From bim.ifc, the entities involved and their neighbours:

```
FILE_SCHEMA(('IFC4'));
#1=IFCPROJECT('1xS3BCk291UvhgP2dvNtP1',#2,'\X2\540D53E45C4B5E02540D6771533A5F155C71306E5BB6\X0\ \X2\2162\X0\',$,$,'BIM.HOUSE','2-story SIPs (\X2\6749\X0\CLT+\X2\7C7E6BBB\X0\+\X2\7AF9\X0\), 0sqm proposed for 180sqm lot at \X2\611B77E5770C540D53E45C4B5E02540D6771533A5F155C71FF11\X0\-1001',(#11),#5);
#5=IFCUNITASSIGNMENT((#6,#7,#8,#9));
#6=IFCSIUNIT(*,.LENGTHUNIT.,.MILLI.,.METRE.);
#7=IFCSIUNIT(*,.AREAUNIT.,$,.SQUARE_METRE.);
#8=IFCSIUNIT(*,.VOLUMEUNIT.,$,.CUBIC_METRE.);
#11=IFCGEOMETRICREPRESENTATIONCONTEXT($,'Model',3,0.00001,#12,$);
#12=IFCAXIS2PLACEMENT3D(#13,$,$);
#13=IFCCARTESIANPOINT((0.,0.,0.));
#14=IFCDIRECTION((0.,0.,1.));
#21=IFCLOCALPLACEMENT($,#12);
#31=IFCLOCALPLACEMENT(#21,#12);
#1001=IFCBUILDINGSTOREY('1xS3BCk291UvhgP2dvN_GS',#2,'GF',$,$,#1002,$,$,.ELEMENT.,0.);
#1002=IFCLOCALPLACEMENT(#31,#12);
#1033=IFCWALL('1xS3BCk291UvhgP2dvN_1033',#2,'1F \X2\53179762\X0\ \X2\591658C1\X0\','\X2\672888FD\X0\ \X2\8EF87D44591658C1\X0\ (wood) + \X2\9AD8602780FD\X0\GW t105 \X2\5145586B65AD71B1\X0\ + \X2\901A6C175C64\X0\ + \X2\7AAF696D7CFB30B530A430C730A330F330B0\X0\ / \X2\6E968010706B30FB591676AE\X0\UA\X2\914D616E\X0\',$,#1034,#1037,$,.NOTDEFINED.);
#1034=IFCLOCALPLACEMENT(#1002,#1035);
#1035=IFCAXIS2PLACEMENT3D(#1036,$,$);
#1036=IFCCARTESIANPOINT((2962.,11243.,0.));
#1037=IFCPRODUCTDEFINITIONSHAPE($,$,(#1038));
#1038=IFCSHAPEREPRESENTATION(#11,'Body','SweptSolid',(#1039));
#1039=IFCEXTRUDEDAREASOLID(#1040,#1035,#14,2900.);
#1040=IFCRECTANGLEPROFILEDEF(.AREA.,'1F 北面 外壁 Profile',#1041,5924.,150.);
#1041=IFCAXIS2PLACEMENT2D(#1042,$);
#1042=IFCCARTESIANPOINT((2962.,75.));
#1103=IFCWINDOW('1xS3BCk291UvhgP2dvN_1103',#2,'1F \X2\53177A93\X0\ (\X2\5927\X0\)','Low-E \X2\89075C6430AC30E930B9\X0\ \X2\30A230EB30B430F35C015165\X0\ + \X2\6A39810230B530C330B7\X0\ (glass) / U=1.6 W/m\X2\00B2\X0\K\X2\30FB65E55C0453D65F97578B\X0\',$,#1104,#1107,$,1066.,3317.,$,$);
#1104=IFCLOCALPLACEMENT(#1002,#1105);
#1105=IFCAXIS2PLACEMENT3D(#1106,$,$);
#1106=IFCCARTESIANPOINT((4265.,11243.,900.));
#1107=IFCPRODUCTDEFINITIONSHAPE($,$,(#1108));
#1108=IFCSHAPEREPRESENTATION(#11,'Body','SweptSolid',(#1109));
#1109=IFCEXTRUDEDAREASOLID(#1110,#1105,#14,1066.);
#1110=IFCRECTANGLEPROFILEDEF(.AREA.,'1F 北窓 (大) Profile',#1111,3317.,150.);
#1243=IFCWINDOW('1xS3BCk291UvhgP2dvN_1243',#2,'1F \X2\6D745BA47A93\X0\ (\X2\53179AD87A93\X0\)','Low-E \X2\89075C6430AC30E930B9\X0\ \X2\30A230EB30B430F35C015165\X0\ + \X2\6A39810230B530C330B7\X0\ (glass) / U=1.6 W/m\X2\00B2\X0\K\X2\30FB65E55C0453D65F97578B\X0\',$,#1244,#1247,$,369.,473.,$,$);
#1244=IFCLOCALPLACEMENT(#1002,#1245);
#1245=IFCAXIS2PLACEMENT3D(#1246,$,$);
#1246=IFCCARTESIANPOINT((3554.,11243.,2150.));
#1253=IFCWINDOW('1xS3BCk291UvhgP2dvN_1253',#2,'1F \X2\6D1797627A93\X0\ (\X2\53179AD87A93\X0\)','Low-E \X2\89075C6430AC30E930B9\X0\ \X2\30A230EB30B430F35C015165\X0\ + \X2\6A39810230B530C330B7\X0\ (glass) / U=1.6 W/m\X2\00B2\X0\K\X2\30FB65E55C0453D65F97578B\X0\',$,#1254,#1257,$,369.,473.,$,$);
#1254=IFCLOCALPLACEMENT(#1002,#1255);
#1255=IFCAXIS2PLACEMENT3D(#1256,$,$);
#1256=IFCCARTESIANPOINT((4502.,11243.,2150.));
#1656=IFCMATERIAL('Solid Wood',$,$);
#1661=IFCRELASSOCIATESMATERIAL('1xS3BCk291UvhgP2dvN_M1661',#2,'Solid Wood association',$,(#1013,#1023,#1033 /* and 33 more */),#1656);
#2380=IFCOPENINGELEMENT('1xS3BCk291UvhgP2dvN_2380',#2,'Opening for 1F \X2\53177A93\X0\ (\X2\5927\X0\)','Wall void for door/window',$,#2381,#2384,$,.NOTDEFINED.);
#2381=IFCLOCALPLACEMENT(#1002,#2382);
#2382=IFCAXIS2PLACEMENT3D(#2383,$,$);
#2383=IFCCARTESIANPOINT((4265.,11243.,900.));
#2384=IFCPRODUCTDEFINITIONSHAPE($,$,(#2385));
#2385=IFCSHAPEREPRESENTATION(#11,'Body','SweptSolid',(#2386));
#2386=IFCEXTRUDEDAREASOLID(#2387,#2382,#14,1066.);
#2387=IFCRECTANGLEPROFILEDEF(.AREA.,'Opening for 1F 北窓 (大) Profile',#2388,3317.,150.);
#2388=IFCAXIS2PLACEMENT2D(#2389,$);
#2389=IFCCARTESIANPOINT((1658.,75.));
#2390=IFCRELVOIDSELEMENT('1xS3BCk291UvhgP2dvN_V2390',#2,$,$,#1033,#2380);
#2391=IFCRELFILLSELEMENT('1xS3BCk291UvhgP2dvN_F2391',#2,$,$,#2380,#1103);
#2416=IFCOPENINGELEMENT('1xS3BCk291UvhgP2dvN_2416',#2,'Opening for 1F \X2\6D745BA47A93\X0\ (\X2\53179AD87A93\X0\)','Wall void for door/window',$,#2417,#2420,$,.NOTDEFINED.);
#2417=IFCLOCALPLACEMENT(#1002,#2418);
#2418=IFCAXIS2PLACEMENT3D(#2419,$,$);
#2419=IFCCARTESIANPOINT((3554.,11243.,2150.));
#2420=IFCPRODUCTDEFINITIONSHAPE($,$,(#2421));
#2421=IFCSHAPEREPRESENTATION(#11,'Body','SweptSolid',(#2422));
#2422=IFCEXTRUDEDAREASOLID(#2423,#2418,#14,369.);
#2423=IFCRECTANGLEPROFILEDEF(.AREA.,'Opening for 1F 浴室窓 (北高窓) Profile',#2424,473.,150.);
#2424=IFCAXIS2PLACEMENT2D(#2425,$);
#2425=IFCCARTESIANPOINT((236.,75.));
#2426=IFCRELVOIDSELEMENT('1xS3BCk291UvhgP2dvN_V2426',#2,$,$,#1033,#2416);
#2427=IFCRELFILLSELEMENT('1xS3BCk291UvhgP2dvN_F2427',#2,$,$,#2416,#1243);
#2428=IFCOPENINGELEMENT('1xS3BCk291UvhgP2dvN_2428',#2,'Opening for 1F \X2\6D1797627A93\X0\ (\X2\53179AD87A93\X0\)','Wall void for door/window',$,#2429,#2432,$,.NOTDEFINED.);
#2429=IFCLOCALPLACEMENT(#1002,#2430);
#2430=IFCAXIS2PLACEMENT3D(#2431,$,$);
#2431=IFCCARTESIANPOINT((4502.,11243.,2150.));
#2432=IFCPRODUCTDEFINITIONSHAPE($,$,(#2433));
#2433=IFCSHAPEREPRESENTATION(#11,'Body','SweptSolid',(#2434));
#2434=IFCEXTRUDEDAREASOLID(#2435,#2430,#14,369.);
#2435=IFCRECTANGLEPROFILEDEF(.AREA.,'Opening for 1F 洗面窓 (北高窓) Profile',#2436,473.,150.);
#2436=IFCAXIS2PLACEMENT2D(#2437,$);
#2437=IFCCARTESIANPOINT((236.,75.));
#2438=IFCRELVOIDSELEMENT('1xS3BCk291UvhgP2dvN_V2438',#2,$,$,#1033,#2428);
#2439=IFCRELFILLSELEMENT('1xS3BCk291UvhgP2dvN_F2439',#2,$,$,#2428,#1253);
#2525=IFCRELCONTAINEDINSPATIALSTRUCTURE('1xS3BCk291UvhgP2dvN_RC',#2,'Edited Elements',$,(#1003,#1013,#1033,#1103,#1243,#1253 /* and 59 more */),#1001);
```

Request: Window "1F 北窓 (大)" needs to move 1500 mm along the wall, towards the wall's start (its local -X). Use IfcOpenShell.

```python
import ifcopenshell
import ifcopenshell.api.geometry
import ifcopenshell.util.placement
import ifcopenshell.util.unit

model = ifcopenshell.open("bim.ifc")
unit_scale = ifcopenshell.util.unit.calculate_unit_scale(model)

window = model.by_guid("1xS3BCk291UvhgP2dvN_1103")
opening = window.FillsVoids[0].RelatingOpeningElement
wall = opening.VoidsElements[0].RelatingBuildingElement

wall_matrix = ifcopenshell.util.placement.get_local_placement(wall.ObjectPlacement)
shift = wall_matrix[:3, 0] * -1.5 / unit_scale
before = ifcopenshell.util.placement.get_local_placement(window.ObjectPlacement)[:3, 3].copy()

# The window is not placed relative to its opening, so move both.
for product in (opening, window):
    matrix = ifcopenshell.util.placement.get_local_placement(product.ObjectPlacement)
    matrix[:3, 3] += shift
    ifcopenshell.api.geometry.edit_object_placement(model, product=product, matrix=matrix, is_si=False)

after = ifcopenshell.util.placement.get_local_placement(window.ObjectPlacement)[:3, 3]
print("window moved by", (after - before).round(3) + 0.0)

model.write("bim_rev.ifc")
```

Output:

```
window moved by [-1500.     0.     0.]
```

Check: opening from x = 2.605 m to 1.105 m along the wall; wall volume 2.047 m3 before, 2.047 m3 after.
